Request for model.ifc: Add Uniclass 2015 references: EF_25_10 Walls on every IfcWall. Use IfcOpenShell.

First a look at what the model holds.

```python
import ifcopenshell

model = ifcopenshell.open("model.ifc")
print(model.schema)
print("classifications:", [c.Name for c in model.by_type("IfcClassification")])
for ifc_class in ("IfcDoor", "IfcRoof", "IfcStair", "IfcWall", "IfcWindow"):
    print(ifc_class, len(model.by_type(ifc_class)))
```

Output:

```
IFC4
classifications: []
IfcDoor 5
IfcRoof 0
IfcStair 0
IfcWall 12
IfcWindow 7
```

```python
import ifcopenshell
import ifcopenshell.api.classification

model = ifcopenshell.open("model.ifc")

system = ifcopenshell.api.classification.add_classification(model, classification="Uniclass 2015")

codes = {
    "IfcWall": ("EF_25_10", "Walls"),
}
for ifc_class, (code, name) in codes.items():
    products = model.by_type(ifc_class)
    ifcopenshell.api.classification.add_reference(
        model, products=products, classification=system, identification=code, name=name
    )
    print(code, len(products))

model.write("model_v2.ifc")
```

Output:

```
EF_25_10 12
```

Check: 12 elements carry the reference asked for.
